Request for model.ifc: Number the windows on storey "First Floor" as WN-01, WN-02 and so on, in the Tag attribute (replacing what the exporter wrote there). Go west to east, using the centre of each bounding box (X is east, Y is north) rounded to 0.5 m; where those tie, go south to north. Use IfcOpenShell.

First a look at what the model holds.

```python
import ifcopenshell
import ifcopenshell.util.element
import ifcopenshell.util.placement

model = ifcopenshell.open("model.ifc")
print(model.schema)
storey = next(s for s in model.by_type("IfcBuildingStorey") if s.Name == "First Floor")
windows = [e for e in ifcopenshell.util.element.get_decomposition(storey) if e.is_a("IfcWindow")]
for e in sorted(windows, key=lambda e: e.id()):
    origin = ifcopenshell.util.placement.get_local_placement(e.ObjectPlacement)[:3, 3]
    print(e.id(), e.Tag, e.Name, origin.round(2) + 0.0, sep=" | ")
```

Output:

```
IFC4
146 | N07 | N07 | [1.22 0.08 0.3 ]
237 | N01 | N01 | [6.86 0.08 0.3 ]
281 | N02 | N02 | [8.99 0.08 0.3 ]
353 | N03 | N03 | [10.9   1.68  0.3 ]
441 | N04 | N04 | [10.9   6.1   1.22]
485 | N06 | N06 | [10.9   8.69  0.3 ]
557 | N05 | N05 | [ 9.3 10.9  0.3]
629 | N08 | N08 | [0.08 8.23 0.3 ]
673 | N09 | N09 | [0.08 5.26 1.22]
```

```python
import ifcopenshell
import ifcopenshell.geom
import ifcopenshell.util.element
import ifcopenshell.util.shape

model = ifcopenshell.open("model.ifc")
settings = ifcopenshell.geom.settings()
settings.set("use-world-coords", True)


def centre(element):
    shape = ifcopenshell.geom.create_shape(settings, element)
    return ifcopenshell.util.shape.get_bbox_centroid(shape.geometry)


storey = next(s for s in model.by_type("IfcBuildingStorey") if s.Name == "First Floor")
windows = [e for e in ifcopenshell.util.element.get_decomposition(storey) if e.is_a("IfcWindow")]

# Insertion points can sit at a corner or the storey origin, so sort by the geometry (in metres).
centres = {e: centre(e) for e in windows}
windows.sort(key=lambda e: (round(centres[e][0] / 0.5), centres[e][1]))

for i, e in enumerate(windows, start=1):
    number = f"WN-{i:02d}"
    e.Tag = number
    print(e.id(), number)

model.write("model-out.ifc")
```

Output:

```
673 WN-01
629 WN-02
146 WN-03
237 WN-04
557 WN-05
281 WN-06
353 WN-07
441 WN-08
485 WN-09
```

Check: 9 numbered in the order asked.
